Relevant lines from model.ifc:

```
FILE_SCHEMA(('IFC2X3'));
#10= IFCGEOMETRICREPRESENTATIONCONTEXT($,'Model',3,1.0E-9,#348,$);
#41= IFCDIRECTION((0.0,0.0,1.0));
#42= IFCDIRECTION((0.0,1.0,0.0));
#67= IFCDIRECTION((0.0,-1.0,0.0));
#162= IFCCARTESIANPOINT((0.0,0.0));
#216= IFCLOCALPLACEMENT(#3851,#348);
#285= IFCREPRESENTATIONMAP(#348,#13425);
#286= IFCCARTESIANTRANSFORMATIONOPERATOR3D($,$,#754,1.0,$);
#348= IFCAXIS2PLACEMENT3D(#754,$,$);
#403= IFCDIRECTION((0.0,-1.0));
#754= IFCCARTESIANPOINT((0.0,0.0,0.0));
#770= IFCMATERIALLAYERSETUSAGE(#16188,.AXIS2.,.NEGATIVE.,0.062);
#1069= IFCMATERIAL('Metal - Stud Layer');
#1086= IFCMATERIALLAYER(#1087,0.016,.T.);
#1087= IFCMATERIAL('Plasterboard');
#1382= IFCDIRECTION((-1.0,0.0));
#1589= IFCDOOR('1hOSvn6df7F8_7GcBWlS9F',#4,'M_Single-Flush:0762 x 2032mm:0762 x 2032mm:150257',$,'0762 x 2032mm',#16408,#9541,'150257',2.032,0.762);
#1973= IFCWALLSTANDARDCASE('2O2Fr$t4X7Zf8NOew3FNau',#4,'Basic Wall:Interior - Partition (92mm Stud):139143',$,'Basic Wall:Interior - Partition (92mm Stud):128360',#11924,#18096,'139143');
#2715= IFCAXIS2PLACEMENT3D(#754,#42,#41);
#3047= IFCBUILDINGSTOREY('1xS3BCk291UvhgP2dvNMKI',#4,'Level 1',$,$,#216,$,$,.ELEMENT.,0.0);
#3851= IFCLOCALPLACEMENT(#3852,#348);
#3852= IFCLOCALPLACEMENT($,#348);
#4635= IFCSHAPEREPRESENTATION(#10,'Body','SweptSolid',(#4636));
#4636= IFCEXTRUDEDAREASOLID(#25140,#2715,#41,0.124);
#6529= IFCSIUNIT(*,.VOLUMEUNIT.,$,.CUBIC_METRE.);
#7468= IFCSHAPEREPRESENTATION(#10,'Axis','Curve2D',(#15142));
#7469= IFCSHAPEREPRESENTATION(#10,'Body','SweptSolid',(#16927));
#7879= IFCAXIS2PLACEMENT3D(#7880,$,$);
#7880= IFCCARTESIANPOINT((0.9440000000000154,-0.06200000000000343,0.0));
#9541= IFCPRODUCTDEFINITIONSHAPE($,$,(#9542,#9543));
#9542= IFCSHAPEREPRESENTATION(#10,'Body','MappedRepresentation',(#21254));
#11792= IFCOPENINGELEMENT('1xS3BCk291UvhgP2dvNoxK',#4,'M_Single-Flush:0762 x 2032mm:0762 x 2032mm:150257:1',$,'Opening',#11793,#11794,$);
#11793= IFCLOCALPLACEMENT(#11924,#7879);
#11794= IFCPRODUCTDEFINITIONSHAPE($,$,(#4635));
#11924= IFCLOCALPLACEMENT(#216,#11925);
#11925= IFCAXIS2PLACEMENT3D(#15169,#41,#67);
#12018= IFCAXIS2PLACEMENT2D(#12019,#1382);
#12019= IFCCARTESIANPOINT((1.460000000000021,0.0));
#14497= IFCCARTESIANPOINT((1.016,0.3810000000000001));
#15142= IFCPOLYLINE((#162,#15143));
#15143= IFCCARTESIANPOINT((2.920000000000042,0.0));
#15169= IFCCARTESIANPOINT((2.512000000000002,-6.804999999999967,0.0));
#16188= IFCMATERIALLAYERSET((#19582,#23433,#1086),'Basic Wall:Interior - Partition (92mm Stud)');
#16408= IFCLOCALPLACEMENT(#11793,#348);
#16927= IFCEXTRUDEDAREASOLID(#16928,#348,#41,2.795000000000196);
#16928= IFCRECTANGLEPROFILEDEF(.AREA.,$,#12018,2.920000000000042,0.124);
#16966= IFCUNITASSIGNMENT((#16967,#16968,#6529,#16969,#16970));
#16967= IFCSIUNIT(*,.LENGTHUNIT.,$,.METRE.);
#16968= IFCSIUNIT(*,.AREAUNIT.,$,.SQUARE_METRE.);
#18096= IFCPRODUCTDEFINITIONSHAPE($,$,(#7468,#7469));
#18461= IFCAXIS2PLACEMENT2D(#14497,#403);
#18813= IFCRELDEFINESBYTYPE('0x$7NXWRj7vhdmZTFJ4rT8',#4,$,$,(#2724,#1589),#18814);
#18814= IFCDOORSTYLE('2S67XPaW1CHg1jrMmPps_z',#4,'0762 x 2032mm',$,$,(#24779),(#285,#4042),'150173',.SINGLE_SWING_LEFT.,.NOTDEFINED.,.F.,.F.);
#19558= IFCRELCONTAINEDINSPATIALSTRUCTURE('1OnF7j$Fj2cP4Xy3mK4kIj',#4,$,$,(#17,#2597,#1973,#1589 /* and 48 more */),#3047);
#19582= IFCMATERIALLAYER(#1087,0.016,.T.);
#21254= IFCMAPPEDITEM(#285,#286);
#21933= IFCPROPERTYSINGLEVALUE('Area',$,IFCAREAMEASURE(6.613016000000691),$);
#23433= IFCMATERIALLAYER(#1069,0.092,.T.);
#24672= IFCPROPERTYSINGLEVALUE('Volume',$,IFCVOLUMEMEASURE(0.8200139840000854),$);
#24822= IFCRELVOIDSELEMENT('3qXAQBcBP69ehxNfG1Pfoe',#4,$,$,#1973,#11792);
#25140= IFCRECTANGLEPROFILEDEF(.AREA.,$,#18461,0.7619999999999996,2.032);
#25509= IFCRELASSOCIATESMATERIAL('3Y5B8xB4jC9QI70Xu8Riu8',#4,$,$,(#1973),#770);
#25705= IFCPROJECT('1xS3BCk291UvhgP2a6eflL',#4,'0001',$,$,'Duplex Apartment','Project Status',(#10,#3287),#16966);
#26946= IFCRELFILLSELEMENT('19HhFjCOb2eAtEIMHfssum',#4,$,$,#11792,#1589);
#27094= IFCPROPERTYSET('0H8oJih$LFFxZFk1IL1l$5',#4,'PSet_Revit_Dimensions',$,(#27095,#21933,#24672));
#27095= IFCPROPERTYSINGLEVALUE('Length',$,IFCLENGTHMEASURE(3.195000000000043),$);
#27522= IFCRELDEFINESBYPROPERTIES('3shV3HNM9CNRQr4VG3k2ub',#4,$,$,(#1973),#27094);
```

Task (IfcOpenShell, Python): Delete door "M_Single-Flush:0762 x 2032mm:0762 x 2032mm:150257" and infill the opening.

```python
import ifcopenshell
import ifcopenshell.api.feature
import ifcopenshell.api.pset
import ifcopenshell.api.root
import ifcopenshell.geom
import ifcopenshell.util.element
import ifcopenshell.util.shape
import ifcopenshell.util.unit

model = ifcopenshell.open("model.ifc")
area_scale = ifcopenshell.util.unit.calculate_unit_scale(model, "AREAUNIT")
volume_scale = ifcopenshell.util.unit.calculate_unit_scale(model, "VOLUMEUNIT")
settings = ifcopenshell.geom.settings()


def volume(element):
    """Net volume in cubic metres, openings subtracted."""
    shape = ifcopenshell.geom.create_shape(settings, element)
    return ifcopenshell.util.shape.get_volume(shape.geometry)


door = model.by_guid("1hOSvn6df7F8_7GcBWlS9F")
opening = door.FillsVoids[0].RelatingOpeningElement
wall = opening.VoidsElements[0].RelatingBuildingElement
before = volume(wall)

ifcopenshell.api.root.remove_product(model, product=door)
ifcopenshell.api.feature.remove_feature(model, feature=opening)

after = volume(wall)
thickness = 0.124  # wall thickness in metres

# Update the wall's stored quantities.
pset = model.by_id(ifcopenshell.util.element.get_pset(wall, "PSet_Revit_Dimensions", should_inherit=False)["id"])
ifcopenshell.api.pset.edit_pset(model, pset=pset, properties={
    "Area": model.create_entity("IfcAreaMeasure", after / thickness / area_scale),
    "Volume": model.create_entity("IfcVolumeMeasure", after / volume_scale),
})

print(f"wall volume {before:.3f} -> {after:.3f} m3")

model.write("model_rev.ifc")
```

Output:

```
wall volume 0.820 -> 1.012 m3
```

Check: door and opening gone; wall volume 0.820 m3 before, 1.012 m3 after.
